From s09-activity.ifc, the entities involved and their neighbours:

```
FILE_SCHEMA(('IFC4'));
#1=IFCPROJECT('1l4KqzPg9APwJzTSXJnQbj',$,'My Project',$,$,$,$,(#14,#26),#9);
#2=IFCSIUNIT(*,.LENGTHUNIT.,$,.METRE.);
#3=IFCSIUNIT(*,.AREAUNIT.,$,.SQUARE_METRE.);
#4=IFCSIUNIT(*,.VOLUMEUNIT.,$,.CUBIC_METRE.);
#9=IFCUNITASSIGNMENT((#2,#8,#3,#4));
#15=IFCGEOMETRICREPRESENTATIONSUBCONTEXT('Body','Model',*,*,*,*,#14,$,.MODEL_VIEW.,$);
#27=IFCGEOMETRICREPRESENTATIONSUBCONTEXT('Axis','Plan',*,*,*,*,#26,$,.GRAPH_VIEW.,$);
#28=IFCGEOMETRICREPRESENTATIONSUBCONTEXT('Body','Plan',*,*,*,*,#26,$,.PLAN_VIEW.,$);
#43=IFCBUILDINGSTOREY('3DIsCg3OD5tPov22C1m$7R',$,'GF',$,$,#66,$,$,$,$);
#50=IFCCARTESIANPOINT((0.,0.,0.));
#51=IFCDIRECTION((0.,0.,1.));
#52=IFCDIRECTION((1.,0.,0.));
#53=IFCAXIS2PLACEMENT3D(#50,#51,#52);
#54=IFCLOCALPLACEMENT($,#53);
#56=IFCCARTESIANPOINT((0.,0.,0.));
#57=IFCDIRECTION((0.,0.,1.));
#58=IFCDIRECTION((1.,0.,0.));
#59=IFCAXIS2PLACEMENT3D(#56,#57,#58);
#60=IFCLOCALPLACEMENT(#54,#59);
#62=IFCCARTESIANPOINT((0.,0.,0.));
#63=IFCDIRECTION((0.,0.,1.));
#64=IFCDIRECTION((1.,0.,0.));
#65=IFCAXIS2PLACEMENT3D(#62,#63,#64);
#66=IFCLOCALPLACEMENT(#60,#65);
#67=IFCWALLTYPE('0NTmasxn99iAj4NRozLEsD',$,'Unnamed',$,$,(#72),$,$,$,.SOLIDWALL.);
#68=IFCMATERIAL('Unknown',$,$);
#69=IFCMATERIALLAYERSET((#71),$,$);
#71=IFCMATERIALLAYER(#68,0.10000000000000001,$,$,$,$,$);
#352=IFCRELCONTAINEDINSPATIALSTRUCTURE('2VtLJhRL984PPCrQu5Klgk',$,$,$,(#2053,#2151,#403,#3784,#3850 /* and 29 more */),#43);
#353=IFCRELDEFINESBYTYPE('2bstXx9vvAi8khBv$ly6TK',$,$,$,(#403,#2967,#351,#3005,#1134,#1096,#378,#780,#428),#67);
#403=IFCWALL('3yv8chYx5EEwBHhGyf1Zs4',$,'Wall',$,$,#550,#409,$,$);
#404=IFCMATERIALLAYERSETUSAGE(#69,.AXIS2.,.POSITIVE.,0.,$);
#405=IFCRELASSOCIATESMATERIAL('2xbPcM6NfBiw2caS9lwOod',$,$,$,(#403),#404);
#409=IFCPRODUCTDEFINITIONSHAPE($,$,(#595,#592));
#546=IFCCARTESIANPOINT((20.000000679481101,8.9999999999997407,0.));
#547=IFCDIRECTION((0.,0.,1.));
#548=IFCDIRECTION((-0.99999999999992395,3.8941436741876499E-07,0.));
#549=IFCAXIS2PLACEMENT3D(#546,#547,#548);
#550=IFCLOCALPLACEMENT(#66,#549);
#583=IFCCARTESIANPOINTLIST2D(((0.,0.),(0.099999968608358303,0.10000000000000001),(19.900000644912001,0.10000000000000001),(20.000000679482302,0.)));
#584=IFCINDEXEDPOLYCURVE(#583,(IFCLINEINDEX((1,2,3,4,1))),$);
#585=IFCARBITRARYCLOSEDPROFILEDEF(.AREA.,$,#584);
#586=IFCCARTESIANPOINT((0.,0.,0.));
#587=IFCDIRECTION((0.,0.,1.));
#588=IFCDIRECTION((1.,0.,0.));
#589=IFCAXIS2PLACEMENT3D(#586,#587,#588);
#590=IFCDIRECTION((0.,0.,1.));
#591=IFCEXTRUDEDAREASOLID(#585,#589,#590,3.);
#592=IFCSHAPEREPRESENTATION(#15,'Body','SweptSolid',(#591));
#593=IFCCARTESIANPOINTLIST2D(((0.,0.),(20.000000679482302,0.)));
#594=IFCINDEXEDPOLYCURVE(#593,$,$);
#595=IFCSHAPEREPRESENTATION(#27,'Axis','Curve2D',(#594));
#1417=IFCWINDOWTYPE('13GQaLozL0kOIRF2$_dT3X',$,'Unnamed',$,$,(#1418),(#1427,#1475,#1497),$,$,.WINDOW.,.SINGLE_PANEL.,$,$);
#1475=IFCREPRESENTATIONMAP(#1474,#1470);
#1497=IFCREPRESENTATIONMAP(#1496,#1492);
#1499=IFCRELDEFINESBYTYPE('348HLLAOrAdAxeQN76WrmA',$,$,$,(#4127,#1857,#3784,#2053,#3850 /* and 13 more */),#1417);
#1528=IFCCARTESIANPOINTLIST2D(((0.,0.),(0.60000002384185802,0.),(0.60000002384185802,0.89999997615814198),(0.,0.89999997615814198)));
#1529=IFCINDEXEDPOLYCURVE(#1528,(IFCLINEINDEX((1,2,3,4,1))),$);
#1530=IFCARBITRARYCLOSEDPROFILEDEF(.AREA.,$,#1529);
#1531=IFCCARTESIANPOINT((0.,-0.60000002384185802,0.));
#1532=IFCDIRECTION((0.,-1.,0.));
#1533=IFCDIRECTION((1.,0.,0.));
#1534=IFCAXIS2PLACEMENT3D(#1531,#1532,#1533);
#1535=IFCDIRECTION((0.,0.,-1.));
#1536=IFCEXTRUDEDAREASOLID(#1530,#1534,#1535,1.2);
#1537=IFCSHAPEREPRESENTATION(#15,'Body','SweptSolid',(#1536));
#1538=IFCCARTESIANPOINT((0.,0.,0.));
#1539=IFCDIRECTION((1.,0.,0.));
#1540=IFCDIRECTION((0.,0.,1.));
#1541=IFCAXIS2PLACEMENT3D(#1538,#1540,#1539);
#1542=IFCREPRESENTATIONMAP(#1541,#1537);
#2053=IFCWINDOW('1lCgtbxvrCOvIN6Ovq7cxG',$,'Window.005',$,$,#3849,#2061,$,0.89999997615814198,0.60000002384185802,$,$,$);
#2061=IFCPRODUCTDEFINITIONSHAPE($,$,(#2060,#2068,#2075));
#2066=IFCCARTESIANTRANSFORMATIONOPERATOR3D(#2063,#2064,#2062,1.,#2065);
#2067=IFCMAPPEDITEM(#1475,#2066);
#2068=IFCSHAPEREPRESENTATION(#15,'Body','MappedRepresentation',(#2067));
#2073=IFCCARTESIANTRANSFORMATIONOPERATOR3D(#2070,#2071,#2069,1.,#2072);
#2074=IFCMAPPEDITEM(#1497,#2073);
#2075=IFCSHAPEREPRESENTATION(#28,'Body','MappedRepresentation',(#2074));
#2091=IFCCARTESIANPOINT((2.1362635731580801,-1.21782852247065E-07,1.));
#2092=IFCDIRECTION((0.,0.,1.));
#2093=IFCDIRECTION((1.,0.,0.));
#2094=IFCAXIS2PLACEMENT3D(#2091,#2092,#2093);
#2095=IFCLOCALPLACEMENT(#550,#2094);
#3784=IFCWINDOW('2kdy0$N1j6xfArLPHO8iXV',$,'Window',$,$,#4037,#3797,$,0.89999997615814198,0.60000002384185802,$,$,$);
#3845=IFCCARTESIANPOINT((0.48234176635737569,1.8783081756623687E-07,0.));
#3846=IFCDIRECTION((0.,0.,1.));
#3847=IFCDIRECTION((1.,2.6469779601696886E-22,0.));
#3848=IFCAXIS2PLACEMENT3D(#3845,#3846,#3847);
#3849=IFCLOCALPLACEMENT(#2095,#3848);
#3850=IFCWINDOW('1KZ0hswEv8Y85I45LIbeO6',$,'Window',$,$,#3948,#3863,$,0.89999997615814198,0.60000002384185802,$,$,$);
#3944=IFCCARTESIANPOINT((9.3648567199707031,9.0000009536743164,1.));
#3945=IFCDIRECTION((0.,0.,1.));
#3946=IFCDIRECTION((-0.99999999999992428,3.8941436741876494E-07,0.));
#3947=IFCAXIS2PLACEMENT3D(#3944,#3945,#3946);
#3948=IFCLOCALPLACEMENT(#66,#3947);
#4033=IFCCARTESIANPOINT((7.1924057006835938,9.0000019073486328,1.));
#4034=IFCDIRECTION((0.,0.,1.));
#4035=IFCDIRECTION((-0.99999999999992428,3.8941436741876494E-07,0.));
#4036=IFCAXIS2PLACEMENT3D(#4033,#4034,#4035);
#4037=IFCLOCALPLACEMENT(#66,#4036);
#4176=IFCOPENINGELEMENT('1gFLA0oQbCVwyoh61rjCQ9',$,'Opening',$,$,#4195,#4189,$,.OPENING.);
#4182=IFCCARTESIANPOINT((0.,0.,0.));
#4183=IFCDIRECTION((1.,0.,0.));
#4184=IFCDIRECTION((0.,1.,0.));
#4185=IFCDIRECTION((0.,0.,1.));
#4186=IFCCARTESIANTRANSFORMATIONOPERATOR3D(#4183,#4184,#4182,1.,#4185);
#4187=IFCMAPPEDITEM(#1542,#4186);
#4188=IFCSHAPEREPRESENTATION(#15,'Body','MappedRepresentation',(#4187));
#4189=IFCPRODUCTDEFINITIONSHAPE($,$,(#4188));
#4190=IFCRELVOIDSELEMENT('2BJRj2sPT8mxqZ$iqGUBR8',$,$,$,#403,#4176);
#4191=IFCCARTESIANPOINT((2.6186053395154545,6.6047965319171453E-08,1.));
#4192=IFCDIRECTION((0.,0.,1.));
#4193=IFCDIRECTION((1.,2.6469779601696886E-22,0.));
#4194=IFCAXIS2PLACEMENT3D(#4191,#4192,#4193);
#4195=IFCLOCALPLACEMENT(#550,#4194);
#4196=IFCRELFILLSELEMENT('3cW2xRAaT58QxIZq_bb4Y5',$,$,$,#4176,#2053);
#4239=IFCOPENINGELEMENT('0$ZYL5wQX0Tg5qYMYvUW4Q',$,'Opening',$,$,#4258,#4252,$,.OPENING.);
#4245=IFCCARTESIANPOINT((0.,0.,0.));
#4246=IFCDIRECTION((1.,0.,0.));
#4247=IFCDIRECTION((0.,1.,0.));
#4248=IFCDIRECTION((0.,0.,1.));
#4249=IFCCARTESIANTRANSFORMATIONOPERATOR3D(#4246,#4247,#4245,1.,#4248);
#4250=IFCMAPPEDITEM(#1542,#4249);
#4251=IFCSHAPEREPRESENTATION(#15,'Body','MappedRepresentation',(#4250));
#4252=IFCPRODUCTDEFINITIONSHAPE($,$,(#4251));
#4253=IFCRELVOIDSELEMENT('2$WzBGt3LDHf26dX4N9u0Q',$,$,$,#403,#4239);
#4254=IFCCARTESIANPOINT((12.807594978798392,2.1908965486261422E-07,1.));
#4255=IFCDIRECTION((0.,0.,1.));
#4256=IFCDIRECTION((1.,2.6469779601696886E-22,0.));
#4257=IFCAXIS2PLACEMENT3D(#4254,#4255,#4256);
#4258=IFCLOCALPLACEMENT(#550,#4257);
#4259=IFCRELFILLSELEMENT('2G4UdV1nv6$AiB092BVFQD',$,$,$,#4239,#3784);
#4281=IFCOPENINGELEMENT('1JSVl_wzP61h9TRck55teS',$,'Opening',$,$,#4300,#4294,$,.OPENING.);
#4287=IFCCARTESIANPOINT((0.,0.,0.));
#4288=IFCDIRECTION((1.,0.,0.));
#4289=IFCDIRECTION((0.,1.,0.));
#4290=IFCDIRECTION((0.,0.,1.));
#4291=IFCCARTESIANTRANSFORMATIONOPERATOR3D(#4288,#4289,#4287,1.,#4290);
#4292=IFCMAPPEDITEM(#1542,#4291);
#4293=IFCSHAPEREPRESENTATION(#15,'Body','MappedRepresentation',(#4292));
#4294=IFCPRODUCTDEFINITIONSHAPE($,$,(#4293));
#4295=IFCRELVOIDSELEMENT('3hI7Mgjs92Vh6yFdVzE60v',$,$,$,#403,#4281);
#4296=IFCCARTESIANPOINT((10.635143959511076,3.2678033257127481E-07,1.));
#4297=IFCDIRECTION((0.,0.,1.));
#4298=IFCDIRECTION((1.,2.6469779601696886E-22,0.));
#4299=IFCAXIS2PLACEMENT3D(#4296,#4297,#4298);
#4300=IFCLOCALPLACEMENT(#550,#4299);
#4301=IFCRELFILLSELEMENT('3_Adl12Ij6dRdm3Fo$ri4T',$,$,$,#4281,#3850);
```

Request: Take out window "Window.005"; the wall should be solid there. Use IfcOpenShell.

```python
import ifcopenshell
import ifcopenshell.api.feature
import ifcopenshell.api.root
import ifcopenshell.geom
import ifcopenshell.util.shape

model = ifcopenshell.open("s09-activity.ifc")
settings = ifcopenshell.geom.settings()


def volume(element):
    """Net volume in cubic metres, openings subtracted."""
    shape = ifcopenshell.geom.create_shape(settings, element)
    return ifcopenshell.util.shape.get_volume(shape.geometry)


window = model.by_guid("1lCgtbxvrCOvIN6Ovq7cxG")
opening = window.FillsVoids[0].RelatingOpeningElement
wall = opening.VoidsElements[0].RelatingBuildingElement
before = volume(wall)

ifcopenshell.api.root.remove_product(model, product=window)
ifcopenshell.api.feature.remove_feature(model, feature=opening)

after = volume(wall)

print(f"wall volume {before:.3f} -> {after:.3f} m3")

model.write("s09-activity_rev.ifc")
```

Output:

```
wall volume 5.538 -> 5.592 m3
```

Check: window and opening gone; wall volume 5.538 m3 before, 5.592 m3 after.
